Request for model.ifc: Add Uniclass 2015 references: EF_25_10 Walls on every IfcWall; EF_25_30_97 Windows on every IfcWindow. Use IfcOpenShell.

First a look at what the model holds.

```python
import ifcopenshell

model = ifcopenshell.open("model.ifc")
print(model.schema)
print("classifications:", [c.Name for c in model.by_type("IfcClassification")])
for ifc_class in ("IfcDoor", "IfcRoof", "IfcStair", "IfcWall", "IfcWindow"):
    print(ifc_class, len(model.by_type(ifc_class)))
```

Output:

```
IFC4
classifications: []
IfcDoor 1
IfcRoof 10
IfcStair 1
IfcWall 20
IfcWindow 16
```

```python
import ifcopenshell
import ifcopenshell.api.classification

model = ifcopenshell.open("model.ifc")

system = ifcopenshell.api.classification.add_classification(model, classification="Uniclass 2015")

codes = {
    "IfcWall": ("EF_25_10", "Walls"),
    "IfcWindow": ("EF_25_30_97", "Windows"),
}
for ifc_class, (code, name) in codes.items():
    products = model.by_type(ifc_class)
    ifcopenshell.api.classification.add_reference(
        model, products=products, classification=system, identification=code, name=name
    )
    print(code, len(products))

model.write("model_rev.ifc")
```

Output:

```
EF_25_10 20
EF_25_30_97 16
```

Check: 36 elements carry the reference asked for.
